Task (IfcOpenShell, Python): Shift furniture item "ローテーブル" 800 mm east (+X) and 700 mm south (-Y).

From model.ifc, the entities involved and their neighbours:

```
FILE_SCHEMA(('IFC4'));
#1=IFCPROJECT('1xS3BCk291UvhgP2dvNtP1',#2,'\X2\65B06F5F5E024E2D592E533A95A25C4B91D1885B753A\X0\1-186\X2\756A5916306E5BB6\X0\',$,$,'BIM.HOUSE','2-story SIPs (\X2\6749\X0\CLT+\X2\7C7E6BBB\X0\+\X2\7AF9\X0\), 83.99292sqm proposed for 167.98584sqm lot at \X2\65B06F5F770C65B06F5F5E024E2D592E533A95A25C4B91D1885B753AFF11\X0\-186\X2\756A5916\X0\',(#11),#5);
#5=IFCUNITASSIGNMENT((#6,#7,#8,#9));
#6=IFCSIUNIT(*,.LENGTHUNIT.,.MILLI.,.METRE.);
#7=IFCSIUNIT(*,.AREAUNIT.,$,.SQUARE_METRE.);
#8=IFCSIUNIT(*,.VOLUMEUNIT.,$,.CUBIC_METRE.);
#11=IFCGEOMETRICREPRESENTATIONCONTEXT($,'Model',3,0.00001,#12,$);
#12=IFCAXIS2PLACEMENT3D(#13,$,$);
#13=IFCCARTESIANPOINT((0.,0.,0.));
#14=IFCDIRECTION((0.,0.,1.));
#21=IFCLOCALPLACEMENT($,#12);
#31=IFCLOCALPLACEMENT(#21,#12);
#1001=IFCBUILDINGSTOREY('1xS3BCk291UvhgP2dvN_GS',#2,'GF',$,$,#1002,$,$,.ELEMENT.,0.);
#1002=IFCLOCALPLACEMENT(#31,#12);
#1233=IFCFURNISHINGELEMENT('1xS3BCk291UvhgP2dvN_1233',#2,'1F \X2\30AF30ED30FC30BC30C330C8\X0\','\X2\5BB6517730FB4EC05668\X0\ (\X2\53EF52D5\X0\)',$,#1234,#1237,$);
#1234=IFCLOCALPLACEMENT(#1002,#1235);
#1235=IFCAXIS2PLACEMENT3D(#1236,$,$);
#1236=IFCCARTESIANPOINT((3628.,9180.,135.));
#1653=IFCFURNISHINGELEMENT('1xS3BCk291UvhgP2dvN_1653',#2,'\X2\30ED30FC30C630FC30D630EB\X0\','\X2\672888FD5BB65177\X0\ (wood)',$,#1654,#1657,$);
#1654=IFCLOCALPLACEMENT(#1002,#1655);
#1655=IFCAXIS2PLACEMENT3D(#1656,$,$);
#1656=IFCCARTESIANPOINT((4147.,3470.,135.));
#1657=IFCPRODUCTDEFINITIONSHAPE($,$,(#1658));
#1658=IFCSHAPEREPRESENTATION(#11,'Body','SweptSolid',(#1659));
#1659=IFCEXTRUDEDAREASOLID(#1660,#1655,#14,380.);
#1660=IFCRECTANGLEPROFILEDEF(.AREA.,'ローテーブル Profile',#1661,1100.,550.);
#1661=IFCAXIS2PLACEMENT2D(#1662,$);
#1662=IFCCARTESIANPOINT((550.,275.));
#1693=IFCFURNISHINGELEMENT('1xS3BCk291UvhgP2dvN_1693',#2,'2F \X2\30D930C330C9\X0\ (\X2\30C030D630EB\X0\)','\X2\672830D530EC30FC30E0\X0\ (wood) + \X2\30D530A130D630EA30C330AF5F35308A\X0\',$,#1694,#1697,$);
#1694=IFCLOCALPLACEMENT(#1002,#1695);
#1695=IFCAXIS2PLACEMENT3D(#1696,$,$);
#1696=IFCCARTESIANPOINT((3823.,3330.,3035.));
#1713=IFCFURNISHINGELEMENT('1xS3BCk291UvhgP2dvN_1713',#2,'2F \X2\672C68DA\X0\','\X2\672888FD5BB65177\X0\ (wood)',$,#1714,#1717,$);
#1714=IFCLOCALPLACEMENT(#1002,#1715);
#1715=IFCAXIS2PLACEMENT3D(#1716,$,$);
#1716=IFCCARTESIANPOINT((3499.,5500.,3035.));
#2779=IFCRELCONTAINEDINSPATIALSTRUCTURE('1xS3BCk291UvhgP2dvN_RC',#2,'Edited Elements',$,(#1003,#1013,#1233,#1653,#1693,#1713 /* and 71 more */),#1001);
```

```python
import ifcopenshell
import ifcopenshell.api.geometry
import ifcopenshell.util.placement
import ifcopenshell.util.unit

model = ifcopenshell.open("model.ifc")
unit_scale = ifcopenshell.util.unit.calculate_unit_scale(model)

item = model.by_guid("1xS3BCk291UvhgP2dvN_1653")
matrix = ifcopenshell.util.placement.get_local_placement(item.ObjectPlacement)
matrix[0, 3] += 0.8 / unit_scale
matrix[1, 3] -= 0.7 / unit_scale
ifcopenshell.api.geometry.edit_object_placement(model, product=item, matrix=matrix, is_si=False)

print(ifcopenshell.util.placement.get_local_placement(item.ObjectPlacement).round(3) + 0.0)

model.write("model_updated.ifc")
```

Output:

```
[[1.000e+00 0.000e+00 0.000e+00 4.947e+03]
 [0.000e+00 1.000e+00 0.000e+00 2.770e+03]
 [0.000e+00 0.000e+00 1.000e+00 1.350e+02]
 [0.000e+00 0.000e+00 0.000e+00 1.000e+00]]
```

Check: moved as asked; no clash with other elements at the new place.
